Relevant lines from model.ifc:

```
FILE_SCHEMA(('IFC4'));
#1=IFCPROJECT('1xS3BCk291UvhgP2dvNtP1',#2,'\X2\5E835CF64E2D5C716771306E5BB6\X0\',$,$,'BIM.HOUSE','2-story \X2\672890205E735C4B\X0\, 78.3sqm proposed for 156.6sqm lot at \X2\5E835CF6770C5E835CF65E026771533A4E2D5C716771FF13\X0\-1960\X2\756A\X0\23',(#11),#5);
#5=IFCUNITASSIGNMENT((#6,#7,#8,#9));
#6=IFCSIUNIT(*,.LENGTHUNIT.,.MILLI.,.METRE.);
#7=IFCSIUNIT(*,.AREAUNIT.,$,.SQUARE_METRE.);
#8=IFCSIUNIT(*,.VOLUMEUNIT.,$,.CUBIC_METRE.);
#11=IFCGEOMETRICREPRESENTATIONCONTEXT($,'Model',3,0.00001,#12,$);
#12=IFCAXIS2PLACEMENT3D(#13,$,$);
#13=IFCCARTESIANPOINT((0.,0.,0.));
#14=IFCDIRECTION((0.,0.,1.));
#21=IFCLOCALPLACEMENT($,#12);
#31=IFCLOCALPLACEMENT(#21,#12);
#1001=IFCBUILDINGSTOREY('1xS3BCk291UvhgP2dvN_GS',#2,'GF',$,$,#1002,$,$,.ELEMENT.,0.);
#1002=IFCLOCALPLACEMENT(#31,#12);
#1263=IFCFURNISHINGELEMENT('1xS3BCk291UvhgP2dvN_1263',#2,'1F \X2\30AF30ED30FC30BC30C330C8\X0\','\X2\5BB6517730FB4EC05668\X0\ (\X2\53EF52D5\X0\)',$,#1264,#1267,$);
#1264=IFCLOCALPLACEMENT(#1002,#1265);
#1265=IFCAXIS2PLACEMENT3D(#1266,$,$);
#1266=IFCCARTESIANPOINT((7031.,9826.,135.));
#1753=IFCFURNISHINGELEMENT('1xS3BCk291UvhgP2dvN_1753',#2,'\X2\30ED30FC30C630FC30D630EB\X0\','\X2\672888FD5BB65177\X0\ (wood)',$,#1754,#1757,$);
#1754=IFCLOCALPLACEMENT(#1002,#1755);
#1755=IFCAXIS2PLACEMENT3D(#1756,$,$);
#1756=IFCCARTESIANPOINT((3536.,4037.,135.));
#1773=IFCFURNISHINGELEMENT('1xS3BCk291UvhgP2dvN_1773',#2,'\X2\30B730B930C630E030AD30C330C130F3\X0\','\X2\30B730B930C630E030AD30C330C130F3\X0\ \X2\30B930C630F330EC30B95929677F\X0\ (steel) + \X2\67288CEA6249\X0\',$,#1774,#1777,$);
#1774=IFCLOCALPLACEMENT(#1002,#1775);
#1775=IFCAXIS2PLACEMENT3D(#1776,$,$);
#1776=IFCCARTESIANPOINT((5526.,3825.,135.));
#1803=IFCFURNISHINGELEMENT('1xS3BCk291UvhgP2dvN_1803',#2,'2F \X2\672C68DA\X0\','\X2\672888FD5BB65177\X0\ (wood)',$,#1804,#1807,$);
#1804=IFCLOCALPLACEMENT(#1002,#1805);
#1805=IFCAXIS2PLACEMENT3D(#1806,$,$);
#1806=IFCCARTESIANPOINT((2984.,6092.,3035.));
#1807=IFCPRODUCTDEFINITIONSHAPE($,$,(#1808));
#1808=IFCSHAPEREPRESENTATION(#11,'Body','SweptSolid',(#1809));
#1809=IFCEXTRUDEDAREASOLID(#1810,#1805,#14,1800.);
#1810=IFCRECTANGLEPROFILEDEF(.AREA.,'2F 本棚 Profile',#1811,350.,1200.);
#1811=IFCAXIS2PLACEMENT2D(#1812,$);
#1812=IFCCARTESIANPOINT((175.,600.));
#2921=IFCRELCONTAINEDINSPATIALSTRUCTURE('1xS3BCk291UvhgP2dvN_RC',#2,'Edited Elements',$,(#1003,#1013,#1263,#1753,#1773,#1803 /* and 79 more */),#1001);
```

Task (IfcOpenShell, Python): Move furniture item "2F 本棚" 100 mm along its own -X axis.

```python
import ifcopenshell
import ifcopenshell.api.geometry
import ifcopenshell.util.placement

model = ifcopenshell.open("model.ifc")

item = model.by_guid("1xS3BCk291UvhgP2dvN_1803")
matrix = ifcopenshell.util.placement.get_local_placement(item.ObjectPlacement)
matrix[:3, 3] -= matrix[:3, 0] * 100.0
ifcopenshell.api.geometry.edit_object_placement(model, product=item, matrix=matrix, is_si=False)

print(ifcopenshell.util.placement.get_local_placement(item.ObjectPlacement).round(3) + 0.0)

model.write("model_rev.ifc")
```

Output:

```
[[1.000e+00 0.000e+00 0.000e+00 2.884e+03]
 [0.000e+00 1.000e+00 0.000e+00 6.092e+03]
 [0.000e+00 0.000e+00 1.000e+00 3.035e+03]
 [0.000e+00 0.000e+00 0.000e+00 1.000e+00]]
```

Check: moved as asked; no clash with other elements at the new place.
